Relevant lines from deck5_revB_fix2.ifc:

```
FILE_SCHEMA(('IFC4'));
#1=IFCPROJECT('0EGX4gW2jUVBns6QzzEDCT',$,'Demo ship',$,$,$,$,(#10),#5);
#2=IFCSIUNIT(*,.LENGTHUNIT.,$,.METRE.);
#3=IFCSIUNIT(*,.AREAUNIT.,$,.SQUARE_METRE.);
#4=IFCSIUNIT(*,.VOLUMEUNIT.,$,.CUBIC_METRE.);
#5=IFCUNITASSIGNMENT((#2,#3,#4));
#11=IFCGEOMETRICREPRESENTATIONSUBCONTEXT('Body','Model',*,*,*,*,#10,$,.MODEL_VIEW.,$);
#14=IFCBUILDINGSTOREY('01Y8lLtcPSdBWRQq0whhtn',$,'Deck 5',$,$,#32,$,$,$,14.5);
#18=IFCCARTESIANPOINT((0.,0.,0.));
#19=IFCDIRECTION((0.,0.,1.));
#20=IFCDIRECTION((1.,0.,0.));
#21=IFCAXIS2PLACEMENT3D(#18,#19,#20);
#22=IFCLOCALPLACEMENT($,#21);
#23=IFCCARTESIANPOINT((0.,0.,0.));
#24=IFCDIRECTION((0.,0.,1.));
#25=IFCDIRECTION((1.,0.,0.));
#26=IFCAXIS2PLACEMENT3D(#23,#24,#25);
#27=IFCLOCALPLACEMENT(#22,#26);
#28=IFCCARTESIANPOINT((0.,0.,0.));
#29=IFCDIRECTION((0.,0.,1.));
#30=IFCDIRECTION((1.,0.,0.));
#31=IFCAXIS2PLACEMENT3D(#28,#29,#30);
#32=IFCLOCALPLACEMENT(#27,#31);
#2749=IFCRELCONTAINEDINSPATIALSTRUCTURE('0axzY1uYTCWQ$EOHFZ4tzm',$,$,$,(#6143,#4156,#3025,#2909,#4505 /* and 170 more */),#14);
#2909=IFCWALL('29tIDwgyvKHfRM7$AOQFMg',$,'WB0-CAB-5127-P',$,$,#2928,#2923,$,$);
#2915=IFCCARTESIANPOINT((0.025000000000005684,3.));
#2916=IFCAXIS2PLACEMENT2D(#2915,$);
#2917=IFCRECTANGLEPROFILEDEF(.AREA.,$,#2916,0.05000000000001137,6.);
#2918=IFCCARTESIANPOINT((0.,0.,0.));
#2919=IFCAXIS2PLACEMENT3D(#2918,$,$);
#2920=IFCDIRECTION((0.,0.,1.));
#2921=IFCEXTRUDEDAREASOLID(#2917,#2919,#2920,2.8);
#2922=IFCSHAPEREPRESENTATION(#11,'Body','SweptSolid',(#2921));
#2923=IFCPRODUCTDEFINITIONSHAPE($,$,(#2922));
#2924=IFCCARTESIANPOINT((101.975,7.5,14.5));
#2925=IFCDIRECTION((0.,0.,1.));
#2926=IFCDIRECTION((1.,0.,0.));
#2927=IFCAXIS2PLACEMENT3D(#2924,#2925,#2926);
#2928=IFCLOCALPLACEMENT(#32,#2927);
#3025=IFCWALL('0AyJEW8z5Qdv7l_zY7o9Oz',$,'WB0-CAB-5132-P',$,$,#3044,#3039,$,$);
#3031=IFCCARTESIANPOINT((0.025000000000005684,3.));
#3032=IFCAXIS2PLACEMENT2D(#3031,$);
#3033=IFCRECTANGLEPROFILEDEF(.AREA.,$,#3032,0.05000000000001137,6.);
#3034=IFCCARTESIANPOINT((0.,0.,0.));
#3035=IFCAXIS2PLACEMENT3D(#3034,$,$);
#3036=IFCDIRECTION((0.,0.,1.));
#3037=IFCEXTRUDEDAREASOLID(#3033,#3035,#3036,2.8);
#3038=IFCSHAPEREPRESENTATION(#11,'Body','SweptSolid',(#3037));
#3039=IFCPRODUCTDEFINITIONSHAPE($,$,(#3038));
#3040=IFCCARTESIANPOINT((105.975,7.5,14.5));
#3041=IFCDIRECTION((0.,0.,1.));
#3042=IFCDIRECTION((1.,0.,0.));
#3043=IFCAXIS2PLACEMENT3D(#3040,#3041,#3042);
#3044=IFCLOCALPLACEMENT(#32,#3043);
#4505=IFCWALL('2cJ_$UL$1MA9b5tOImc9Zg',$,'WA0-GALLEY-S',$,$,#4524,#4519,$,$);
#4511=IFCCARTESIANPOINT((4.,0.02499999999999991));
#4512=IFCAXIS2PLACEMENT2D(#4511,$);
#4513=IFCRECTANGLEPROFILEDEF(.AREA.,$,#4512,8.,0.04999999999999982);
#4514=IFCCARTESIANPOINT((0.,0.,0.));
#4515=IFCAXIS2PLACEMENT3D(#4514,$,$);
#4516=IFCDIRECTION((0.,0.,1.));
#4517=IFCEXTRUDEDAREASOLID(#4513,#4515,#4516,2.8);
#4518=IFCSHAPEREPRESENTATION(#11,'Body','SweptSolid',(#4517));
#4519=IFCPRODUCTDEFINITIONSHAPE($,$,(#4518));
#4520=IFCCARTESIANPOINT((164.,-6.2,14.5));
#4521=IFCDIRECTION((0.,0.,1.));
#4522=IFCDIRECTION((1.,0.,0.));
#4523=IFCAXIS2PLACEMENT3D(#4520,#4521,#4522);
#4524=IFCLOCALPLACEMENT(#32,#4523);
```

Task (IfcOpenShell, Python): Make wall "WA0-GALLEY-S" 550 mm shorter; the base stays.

```python
import ifcopenshell
import ifcopenshell.geom
import ifcopenshell.util.representation
import ifcopenshell.util.shape
import ifcopenshell.util.unit

model = ifcopenshell.open("deck5_revB_fix2.ifc")
unit_scale = ifcopenshell.util.unit.calculate_unit_scale(model)
settings = ifcopenshell.geom.settings()


def volume(element):
    """Net volume in cubic metres, openings subtracted."""
    shape = ifcopenshell.geom.create_shape(settings, element)
    return ifcopenshell.util.shape.get_volume(shape.geometry)


wall = model.by_guid("2cJ_$UL$1MA9b5tOImc9Zg")
before = volume(wall)

body = ifcopenshell.util.representation.get_representation(wall, "Model", "Body")
solid = body.Items[0]
old_height = solid.Depth
solid.Depth -= 0.55 / unit_scale
after = volume(wall)

print(f"height {old_height:g} -> {solid.Depth:g}, volume {before:.3f} -> {after:.3f} m3")

model.write("deck5_revB_fix2_rev.ifc")
```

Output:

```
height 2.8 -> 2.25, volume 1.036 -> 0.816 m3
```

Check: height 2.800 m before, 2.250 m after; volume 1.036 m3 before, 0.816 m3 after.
